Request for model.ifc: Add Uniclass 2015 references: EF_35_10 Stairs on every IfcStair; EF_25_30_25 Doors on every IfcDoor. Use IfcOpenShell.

First a look at what the model holds.

```python
import ifcopenshell

model = ifcopenshell.open("model.ifc")
print(model.schema)
print("classifications:", [c.Name for c in model.by_type("IfcClassification")])
for ifc_class in ("IfcDoor", "IfcRoof", "IfcStair", "IfcWall", "IfcWindow"):
    print(ifc_class, len(model.by_type(ifc_class)))
```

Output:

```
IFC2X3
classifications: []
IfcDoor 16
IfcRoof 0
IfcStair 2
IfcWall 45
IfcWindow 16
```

```python
import ifcopenshell
import ifcopenshell.api.classification

model = ifcopenshell.open("model.ifc")

# IFC2X3 requires Source and Edition and has no link from the project to the system.
system = model.create_entity("IfcClassification", Source="NBS", Edition="2015", Name="Uniclass 2015")

codes = {
    "IfcStair": ("EF_35_10", "Stairs"),
    "IfcDoor": ("EF_25_30_25", "Doors"),
}
for ifc_class, (code, name) in codes.items():
    products = model.by_type(ifc_class)
    ifcopenshell.api.classification.add_reference(
        model, products=products, classification=system, identification=code, name=name
    )
    print(code, len(products))

model.write("model-out.ifc")
```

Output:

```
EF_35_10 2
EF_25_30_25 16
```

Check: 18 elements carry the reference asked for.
